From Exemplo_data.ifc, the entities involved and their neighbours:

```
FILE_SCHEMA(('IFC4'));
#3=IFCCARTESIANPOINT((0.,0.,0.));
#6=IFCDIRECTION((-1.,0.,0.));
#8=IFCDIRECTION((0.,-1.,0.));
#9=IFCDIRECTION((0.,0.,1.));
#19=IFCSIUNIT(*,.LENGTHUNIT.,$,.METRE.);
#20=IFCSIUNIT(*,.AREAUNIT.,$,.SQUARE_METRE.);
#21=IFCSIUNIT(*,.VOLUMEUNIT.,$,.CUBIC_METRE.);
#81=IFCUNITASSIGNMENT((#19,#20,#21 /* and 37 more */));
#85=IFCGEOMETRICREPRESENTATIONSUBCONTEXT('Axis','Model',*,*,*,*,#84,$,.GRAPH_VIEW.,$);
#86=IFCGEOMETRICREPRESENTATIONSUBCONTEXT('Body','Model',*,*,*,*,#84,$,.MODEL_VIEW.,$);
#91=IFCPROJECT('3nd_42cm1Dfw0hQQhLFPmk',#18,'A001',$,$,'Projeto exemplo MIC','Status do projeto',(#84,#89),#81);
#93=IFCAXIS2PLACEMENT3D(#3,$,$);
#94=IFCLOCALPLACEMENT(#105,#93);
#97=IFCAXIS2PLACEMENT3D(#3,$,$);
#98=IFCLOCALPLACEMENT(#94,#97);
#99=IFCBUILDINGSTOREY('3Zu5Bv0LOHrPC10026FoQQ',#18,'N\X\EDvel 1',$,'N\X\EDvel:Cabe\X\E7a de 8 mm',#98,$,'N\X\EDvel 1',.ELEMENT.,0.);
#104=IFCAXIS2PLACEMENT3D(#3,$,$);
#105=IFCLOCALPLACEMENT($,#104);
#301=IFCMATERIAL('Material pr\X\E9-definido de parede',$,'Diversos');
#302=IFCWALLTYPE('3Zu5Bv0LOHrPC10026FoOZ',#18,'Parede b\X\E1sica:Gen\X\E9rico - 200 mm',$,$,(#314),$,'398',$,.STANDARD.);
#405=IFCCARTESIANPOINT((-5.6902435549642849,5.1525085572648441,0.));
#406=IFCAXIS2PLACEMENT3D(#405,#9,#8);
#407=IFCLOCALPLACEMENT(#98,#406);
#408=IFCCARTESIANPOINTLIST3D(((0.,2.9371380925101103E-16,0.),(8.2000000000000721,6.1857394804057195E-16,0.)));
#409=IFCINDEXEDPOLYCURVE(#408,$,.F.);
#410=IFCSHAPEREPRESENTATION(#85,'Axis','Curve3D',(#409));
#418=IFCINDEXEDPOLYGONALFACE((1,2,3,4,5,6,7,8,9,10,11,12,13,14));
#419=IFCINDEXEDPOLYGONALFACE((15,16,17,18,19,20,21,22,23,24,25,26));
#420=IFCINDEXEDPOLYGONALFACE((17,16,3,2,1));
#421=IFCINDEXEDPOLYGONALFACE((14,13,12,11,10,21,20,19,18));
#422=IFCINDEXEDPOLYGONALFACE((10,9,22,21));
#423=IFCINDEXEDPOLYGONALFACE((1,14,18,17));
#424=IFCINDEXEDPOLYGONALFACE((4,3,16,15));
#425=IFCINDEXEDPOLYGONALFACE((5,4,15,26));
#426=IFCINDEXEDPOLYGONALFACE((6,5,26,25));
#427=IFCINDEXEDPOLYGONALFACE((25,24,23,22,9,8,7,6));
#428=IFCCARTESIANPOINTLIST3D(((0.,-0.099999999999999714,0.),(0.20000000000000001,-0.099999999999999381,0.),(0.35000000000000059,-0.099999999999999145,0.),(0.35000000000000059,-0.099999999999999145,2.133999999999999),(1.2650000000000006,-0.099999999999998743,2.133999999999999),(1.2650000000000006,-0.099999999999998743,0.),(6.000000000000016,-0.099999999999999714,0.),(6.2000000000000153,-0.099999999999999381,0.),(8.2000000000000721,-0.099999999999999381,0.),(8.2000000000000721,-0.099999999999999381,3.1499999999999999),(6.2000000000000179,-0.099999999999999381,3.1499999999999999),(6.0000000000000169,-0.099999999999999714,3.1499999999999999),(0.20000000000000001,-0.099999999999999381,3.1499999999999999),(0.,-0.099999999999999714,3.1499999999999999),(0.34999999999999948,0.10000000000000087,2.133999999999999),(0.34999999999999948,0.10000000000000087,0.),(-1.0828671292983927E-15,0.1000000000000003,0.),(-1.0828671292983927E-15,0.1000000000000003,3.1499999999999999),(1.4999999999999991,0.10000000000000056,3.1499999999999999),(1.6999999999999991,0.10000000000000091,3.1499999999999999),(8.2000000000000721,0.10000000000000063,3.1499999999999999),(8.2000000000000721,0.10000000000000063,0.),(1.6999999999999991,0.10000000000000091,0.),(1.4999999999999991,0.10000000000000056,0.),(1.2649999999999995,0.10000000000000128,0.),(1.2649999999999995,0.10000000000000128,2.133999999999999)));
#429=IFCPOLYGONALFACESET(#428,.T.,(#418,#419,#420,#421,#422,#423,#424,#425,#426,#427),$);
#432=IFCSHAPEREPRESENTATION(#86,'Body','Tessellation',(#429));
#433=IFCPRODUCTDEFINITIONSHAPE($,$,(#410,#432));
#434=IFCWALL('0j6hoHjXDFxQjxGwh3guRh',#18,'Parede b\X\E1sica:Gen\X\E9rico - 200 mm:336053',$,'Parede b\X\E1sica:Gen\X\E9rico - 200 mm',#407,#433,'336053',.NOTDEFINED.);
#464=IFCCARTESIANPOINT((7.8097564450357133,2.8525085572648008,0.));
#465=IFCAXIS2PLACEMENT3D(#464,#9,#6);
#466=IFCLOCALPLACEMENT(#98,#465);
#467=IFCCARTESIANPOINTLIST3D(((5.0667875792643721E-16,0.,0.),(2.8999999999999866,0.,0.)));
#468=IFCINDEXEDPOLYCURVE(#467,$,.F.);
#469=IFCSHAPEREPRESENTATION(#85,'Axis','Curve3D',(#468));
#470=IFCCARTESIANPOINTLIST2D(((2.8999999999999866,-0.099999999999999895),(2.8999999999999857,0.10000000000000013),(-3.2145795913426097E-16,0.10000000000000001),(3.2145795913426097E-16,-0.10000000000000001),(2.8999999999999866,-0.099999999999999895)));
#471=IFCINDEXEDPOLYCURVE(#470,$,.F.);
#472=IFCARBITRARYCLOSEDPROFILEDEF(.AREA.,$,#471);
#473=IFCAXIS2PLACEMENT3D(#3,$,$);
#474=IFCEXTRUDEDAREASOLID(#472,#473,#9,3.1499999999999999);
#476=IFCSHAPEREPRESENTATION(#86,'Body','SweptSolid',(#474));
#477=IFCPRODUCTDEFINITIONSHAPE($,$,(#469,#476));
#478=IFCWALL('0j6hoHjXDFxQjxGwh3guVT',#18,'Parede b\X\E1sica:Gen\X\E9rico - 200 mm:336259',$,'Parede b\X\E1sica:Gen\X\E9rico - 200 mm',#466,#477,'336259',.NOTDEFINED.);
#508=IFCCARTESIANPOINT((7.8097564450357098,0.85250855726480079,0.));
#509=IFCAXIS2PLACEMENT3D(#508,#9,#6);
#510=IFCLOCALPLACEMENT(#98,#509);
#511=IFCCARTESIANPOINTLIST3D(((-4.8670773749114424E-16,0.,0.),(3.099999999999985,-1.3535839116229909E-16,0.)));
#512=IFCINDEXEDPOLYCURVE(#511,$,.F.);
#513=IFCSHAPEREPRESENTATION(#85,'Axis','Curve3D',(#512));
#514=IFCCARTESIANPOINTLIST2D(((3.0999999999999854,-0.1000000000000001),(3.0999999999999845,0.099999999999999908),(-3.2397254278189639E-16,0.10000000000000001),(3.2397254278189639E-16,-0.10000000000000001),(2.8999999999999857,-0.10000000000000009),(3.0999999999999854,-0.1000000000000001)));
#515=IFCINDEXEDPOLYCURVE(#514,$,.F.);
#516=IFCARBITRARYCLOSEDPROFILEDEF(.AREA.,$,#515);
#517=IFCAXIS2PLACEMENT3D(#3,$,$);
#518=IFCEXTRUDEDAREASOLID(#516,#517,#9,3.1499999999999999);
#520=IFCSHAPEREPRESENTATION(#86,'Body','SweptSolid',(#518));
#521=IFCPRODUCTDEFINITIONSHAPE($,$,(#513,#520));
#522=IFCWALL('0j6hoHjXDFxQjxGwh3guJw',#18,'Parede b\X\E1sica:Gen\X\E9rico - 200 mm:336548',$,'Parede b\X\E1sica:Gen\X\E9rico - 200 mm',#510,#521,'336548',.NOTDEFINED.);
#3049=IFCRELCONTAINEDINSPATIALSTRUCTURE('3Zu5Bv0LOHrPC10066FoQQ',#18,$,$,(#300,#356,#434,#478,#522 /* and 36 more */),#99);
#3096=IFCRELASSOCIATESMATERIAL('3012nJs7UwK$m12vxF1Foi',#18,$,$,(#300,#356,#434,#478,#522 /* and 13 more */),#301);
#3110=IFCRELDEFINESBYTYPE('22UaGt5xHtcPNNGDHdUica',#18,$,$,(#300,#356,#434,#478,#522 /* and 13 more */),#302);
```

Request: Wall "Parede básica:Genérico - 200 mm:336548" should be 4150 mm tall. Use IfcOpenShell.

```python
import ifcopenshell
import ifcopenshell.geom
import ifcopenshell.util.representation
import ifcopenshell.util.shape
import ifcopenshell.util.unit

model = ifcopenshell.open("Exemplo_data.ifc")
unit_scale = ifcopenshell.util.unit.calculate_unit_scale(model)
settings = ifcopenshell.geom.settings()


def volume(element):
    """Net volume in cubic metres, openings subtracted."""
    shape = ifcopenshell.geom.create_shape(settings, element)
    return ifcopenshell.util.shape.get_volume(shape.geometry)


wall = model.by_guid("0j6hoHjXDFxQjxGwh3guJw")
before = volume(wall)

body = ifcopenshell.util.representation.get_representation(wall, "Model", "Body")
solid = body.Items[0]
old_height = solid.Depth
solid.Depth = 4.15 / unit_scale
after = volume(wall)

print(f"height {old_height:g} -> {solid.Depth:g}, volume {before:.3f} -> {after:.3f} m3")

model.write("Exemplo_data-out.ifc")
```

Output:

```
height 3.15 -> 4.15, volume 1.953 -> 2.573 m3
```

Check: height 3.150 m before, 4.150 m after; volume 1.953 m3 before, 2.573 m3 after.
